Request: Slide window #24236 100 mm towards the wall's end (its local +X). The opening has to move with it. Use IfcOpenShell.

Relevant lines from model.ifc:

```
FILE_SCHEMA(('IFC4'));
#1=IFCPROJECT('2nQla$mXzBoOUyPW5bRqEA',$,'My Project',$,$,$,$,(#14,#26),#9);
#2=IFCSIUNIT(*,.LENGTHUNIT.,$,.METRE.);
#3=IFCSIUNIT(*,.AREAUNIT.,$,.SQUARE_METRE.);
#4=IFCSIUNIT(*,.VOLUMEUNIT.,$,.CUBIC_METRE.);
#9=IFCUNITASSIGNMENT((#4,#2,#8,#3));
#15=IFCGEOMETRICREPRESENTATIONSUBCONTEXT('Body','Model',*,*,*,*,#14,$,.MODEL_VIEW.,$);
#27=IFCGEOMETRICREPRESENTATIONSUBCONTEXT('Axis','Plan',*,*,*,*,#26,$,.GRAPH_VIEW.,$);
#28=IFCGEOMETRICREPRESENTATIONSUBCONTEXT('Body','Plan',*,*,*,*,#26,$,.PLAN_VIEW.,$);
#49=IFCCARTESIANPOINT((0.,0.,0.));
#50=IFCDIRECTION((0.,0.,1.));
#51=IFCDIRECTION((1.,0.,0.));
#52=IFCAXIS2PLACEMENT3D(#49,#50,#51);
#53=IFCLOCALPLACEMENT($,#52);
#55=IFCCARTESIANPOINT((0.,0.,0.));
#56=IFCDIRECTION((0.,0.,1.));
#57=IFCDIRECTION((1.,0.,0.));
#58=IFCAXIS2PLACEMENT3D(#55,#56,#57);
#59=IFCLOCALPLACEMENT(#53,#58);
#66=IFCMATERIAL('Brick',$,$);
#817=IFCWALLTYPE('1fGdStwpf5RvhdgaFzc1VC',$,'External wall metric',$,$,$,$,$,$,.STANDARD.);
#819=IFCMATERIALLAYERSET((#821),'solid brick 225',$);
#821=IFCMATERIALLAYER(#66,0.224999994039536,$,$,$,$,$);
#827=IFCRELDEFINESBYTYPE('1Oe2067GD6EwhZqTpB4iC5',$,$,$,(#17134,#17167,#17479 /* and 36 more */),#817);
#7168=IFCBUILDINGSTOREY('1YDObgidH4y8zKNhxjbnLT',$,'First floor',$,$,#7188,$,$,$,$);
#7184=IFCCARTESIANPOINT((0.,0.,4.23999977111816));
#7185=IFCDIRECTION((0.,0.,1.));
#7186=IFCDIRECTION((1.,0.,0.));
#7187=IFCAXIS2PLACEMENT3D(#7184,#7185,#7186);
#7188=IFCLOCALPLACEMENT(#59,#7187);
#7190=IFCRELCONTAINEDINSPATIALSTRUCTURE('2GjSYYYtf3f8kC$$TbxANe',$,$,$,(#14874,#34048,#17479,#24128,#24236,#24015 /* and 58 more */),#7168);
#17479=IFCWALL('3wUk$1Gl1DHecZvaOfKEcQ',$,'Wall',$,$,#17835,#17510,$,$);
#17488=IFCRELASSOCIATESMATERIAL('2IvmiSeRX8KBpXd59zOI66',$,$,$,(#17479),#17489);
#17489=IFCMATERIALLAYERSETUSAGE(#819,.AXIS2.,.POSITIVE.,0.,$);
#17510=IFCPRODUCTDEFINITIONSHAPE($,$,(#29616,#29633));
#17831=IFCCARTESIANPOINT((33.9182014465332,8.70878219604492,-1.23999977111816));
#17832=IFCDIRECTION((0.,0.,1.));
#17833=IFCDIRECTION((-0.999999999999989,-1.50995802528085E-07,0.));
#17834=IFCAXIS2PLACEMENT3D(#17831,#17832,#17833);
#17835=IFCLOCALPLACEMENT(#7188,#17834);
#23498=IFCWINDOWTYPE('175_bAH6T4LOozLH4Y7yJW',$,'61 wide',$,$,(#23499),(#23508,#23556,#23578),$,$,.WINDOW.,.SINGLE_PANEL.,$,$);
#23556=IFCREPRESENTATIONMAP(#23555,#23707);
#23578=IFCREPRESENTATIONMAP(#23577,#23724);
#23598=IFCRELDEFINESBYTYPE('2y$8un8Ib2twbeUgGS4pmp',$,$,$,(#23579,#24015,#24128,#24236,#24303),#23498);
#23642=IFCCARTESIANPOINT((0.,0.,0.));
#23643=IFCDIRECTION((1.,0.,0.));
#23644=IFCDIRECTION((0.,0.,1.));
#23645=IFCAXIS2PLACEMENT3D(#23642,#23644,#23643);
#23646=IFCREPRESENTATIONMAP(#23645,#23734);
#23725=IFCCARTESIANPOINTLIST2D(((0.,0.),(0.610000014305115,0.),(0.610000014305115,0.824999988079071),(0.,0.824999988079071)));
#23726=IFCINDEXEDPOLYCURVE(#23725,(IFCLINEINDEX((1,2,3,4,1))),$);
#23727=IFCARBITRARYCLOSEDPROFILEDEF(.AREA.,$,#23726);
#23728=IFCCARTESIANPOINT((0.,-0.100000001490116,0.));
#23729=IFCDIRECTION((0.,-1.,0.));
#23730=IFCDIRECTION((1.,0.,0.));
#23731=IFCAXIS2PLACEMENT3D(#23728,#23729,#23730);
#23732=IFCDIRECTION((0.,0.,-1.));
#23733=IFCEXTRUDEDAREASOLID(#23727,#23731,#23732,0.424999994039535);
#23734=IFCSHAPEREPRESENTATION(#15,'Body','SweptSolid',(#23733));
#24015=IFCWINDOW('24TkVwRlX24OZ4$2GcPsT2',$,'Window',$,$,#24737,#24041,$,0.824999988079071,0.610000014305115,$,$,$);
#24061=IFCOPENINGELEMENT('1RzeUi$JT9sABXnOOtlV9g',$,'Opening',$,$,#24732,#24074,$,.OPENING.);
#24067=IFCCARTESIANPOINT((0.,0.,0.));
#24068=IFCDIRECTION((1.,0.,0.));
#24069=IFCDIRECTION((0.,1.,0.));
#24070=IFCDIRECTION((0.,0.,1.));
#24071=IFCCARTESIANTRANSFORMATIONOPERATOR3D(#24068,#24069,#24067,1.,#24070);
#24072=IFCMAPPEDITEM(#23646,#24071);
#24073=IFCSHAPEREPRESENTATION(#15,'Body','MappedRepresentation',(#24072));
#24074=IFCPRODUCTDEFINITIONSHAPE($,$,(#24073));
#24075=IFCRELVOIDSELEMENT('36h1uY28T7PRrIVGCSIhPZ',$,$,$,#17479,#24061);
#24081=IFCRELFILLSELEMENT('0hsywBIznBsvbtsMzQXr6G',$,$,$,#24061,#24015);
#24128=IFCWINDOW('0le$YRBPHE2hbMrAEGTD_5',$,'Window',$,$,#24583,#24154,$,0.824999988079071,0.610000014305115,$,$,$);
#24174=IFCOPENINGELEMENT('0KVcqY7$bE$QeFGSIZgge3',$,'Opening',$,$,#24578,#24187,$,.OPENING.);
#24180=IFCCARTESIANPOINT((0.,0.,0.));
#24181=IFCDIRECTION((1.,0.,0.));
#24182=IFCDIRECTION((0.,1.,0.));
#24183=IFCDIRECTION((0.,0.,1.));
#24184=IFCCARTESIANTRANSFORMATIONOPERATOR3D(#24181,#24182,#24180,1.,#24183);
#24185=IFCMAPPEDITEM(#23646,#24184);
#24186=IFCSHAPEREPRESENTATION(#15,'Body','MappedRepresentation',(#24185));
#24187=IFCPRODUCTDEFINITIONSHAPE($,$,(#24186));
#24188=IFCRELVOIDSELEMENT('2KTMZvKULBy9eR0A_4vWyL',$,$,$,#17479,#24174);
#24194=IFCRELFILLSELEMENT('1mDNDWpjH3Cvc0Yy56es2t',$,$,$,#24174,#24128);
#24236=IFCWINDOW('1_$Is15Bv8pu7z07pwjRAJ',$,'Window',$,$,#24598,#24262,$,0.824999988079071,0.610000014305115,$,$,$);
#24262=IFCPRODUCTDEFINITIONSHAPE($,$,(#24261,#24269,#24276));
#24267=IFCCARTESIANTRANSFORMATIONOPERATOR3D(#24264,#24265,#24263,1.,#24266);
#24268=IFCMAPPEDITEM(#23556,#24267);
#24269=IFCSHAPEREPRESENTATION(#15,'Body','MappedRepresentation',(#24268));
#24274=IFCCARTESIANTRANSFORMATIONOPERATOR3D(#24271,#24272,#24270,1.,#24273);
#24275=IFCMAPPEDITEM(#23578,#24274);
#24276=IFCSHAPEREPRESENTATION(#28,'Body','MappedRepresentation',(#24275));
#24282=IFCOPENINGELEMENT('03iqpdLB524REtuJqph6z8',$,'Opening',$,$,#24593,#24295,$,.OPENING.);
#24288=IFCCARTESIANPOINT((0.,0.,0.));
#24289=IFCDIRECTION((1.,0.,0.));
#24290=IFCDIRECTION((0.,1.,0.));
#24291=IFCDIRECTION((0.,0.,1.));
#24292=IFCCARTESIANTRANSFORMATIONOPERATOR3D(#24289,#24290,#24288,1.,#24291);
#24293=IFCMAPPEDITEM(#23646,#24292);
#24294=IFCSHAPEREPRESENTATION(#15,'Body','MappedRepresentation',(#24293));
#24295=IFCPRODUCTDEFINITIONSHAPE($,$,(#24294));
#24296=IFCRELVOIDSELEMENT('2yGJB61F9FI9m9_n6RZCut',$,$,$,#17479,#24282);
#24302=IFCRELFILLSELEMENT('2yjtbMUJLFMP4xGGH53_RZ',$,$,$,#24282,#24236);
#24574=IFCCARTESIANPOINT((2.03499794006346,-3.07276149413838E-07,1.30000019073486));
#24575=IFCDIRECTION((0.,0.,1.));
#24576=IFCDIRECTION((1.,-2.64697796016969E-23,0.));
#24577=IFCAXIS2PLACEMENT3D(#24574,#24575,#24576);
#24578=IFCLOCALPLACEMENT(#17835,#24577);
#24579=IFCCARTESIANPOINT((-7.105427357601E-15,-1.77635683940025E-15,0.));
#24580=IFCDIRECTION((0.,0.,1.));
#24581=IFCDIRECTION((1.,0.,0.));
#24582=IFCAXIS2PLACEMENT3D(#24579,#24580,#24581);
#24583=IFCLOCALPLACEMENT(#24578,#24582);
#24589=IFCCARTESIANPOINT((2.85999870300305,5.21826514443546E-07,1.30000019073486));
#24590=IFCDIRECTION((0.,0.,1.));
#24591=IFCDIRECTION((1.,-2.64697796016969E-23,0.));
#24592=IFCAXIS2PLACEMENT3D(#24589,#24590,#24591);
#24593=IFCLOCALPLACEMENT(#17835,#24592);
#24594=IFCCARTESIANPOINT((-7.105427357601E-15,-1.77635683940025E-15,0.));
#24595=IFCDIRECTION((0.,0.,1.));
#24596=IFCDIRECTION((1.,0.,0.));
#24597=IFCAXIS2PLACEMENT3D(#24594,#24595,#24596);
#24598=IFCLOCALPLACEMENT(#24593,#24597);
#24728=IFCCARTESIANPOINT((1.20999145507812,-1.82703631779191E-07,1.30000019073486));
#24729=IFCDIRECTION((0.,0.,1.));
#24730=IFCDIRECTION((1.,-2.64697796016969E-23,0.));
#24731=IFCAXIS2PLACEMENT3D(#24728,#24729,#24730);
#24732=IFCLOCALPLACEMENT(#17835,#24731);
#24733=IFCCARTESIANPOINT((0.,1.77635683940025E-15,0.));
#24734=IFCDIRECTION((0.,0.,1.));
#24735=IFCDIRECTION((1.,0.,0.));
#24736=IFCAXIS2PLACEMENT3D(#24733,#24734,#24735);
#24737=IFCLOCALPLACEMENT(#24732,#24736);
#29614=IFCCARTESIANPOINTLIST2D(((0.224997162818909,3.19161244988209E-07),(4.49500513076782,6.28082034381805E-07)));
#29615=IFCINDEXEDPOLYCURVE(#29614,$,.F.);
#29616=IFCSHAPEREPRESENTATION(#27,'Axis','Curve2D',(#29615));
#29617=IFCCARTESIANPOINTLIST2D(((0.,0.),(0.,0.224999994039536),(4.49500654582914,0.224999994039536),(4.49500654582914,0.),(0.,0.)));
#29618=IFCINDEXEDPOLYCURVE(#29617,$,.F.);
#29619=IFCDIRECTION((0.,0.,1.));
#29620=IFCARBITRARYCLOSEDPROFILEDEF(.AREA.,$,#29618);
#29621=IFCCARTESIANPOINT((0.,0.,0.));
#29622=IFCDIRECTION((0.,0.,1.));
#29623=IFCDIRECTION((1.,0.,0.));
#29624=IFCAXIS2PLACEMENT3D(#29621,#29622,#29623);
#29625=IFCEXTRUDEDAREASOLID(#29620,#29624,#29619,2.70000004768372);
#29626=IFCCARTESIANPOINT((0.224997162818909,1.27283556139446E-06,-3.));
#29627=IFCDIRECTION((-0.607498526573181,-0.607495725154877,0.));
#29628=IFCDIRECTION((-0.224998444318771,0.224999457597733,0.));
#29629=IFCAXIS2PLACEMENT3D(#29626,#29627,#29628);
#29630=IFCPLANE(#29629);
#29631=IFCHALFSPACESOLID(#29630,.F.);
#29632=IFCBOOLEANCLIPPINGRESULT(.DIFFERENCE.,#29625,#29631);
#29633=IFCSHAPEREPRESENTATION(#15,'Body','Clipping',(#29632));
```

```python
import ifcopenshell
import ifcopenshell.api.geometry
import ifcopenshell.util.placement

model = ifcopenshell.open("model.ifc")

window = model.by_guid("1_$Is15Bv8pu7z07pwjRAJ")
opening = window.FillsVoids[0].RelatingOpeningElement
wall = opening.VoidsElements[0].RelatingBuildingElement

wall_matrix = ifcopenshell.util.placement.get_local_placement(wall.ObjectPlacement)
shift = wall_matrix[:3, 0] * 0.1
before = ifcopenshell.util.placement.get_local_placement(window.ObjectPlacement)[:3, 3].copy()

# The window is placed relative to its opening, so it follows when the opening moves.
matrix = ifcopenshell.util.placement.get_local_placement(opening.ObjectPlacement)
matrix[:3, 3] += shift
ifcopenshell.api.geometry.edit_object_placement(
    model, product=opening, matrix=matrix, is_si=False, should_transform_children=True
)

after = ifcopenshell.util.placement.get_local_placement(window.ObjectPlacement)[:3, 3]
print("window moved by", (after - before).round(3) + 0.0)

model.write("model-out.ifc")
```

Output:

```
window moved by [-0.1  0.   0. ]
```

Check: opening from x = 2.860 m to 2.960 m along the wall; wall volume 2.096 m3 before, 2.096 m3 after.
